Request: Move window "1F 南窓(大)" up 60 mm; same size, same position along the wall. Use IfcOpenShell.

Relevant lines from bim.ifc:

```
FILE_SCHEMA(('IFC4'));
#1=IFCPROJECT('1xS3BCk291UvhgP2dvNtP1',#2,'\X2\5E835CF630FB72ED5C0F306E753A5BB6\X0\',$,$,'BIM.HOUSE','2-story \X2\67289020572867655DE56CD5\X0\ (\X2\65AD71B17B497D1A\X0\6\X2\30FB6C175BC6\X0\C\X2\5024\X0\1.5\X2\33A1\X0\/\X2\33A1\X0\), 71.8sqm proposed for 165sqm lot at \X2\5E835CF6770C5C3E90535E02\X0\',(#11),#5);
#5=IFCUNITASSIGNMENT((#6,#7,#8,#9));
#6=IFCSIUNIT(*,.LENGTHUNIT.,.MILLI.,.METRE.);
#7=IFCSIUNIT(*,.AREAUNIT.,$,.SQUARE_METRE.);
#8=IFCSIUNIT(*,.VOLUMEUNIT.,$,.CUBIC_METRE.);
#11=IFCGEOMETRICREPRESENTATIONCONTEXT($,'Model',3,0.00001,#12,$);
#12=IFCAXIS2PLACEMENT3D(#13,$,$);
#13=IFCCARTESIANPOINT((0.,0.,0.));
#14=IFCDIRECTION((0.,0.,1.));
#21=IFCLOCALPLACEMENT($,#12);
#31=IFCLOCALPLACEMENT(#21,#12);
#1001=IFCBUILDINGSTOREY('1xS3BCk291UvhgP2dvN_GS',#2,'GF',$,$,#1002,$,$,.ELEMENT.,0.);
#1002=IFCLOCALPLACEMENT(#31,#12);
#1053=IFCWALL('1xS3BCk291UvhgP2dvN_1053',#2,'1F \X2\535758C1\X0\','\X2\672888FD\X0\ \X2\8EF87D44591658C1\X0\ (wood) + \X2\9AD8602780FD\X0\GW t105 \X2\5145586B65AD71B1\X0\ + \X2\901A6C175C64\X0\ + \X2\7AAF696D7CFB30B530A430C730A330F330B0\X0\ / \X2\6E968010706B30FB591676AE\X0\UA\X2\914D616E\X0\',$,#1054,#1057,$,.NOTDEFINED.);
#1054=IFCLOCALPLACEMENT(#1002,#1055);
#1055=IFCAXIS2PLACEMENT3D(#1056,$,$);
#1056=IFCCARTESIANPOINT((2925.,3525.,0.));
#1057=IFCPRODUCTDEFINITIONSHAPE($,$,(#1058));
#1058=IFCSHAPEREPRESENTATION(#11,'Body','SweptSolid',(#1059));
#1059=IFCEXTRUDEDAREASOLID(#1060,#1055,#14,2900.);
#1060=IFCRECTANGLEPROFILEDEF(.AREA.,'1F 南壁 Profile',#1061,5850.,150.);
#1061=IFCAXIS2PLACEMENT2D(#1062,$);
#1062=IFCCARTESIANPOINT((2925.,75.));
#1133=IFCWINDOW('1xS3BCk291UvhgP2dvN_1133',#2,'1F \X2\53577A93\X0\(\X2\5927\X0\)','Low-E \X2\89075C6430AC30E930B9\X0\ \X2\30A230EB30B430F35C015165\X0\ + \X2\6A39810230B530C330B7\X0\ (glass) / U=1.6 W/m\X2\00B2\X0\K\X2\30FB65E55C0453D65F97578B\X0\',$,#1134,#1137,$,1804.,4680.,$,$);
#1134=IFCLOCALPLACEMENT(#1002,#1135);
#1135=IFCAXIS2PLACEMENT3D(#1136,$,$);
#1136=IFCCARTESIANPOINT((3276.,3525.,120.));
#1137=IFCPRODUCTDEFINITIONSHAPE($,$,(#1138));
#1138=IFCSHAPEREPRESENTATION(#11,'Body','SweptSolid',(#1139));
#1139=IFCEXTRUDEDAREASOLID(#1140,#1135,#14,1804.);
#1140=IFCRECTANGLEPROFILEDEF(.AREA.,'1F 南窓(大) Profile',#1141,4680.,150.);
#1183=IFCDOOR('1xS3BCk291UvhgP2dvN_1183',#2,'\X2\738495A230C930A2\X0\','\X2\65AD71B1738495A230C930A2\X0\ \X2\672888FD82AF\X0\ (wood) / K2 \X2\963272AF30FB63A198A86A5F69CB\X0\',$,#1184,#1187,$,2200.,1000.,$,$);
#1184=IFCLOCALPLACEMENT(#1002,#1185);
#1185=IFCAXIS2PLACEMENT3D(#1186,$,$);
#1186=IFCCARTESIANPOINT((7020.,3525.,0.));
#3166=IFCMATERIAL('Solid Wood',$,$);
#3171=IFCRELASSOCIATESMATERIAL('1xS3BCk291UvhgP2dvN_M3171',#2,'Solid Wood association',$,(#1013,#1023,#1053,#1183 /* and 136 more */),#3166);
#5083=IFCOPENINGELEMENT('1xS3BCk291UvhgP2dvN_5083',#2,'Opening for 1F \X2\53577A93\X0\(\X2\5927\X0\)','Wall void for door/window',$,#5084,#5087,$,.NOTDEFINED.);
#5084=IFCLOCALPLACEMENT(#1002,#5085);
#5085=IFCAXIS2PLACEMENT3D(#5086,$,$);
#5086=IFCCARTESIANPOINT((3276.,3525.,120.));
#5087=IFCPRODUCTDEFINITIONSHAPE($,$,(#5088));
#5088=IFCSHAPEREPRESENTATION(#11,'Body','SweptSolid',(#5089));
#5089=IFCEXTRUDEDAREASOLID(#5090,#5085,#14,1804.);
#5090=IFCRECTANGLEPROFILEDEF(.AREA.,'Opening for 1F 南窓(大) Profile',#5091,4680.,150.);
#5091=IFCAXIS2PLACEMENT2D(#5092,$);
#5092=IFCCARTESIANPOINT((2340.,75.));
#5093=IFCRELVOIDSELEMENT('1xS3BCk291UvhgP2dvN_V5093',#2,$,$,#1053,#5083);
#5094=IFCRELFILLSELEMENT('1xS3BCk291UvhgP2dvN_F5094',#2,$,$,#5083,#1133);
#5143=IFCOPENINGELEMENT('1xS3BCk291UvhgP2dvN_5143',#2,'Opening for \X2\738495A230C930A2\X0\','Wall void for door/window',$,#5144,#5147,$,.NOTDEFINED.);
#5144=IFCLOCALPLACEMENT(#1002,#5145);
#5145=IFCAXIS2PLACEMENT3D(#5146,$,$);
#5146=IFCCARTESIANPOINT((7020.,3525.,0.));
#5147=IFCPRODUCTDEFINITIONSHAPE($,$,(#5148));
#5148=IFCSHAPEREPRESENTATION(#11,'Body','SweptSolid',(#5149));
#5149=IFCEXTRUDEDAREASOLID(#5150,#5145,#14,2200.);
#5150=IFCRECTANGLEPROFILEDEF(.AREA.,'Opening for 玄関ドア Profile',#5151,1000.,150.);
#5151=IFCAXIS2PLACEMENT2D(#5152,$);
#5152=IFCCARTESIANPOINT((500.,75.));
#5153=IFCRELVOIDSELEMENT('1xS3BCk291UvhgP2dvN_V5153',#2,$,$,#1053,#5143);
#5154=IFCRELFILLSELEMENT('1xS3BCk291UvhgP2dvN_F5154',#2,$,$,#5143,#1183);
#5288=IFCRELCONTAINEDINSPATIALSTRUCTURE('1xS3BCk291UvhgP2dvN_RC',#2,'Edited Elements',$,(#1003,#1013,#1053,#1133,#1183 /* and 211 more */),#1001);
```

```python
import numpy as np
import ifcopenshell
import ifcopenshell.api.geometry
import ifcopenshell.util.placement
import ifcopenshell.util.unit

model = ifcopenshell.open("bim.ifc")
unit_scale = ifcopenshell.util.unit.calculate_unit_scale(model)

window = model.by_guid("1xS3BCk291UvhgP2dvN_1133")
opening = window.FillsVoids[0].RelatingOpeningElement
dz = 0.06 / unit_scale

shift = np.array([0.0, 0.0, dz])
# The window is not placed relative to its opening, so move both.
for product in (opening, window):
    matrix = ifcopenshell.util.placement.get_local_placement(product.ObjectPlacement)
    matrix[:3, 3] += shift
    ifcopenshell.api.geometry.edit_object_placement(model, product=product, matrix=matrix, is_si=False)

print(f"moved by {dz * unit_scale:+.3f} m")

model.write("bim_rev.ifc")
```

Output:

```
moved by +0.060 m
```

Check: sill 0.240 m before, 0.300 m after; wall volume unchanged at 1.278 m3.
